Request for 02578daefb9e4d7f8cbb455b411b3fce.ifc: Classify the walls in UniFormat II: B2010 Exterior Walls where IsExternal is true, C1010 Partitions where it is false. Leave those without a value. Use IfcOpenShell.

First a look at what the model holds.

```python
import ifcopenshell
import ifcopenshell.util.element

model = ifcopenshell.open("02578daefb9e4d7f8cbb455b411b3fce.ifc")
print(model.schema)
print("classifications:", [c.Name for c in model.by_type("IfcClassification")])
values = [ifcopenshell.util.element.get_pset(e, "Pset_WallCommon", "IsExternal") for e in model.by_type("IfcWall")]
for value in (True, False, None):
    print("IsExternal", value, values.count(value))
```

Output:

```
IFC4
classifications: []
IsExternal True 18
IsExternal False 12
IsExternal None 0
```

```python
import ifcopenshell
import ifcopenshell.api.classification
import ifcopenshell.util.element

model = ifcopenshell.open("02578daefb9e4d7f8cbb455b411b3fce.ifc")

system = ifcopenshell.api.classification.add_classification(model, classification="UniFormat II")

walls = model.by_type("IfcWall")
external = {e: ifcopenshell.util.element.get_pset(e, "Pset_WallCommon", "IsExternal") for e in walls}
for flag, code, name in ((True, "B2010", "Exterior Walls"), (False, "C1010", "Partitions")):
    products = [e for e in walls if external[e] is flag]
    ifcopenshell.api.classification.add_reference(
        model, products=products, classification=system, identification=code, name=name
    )
    print(code, len(products))

model.write("02578daefb9e4d7f8cbb455b411b3fce_rev.ifc")
```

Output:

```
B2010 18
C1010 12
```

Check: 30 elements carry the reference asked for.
